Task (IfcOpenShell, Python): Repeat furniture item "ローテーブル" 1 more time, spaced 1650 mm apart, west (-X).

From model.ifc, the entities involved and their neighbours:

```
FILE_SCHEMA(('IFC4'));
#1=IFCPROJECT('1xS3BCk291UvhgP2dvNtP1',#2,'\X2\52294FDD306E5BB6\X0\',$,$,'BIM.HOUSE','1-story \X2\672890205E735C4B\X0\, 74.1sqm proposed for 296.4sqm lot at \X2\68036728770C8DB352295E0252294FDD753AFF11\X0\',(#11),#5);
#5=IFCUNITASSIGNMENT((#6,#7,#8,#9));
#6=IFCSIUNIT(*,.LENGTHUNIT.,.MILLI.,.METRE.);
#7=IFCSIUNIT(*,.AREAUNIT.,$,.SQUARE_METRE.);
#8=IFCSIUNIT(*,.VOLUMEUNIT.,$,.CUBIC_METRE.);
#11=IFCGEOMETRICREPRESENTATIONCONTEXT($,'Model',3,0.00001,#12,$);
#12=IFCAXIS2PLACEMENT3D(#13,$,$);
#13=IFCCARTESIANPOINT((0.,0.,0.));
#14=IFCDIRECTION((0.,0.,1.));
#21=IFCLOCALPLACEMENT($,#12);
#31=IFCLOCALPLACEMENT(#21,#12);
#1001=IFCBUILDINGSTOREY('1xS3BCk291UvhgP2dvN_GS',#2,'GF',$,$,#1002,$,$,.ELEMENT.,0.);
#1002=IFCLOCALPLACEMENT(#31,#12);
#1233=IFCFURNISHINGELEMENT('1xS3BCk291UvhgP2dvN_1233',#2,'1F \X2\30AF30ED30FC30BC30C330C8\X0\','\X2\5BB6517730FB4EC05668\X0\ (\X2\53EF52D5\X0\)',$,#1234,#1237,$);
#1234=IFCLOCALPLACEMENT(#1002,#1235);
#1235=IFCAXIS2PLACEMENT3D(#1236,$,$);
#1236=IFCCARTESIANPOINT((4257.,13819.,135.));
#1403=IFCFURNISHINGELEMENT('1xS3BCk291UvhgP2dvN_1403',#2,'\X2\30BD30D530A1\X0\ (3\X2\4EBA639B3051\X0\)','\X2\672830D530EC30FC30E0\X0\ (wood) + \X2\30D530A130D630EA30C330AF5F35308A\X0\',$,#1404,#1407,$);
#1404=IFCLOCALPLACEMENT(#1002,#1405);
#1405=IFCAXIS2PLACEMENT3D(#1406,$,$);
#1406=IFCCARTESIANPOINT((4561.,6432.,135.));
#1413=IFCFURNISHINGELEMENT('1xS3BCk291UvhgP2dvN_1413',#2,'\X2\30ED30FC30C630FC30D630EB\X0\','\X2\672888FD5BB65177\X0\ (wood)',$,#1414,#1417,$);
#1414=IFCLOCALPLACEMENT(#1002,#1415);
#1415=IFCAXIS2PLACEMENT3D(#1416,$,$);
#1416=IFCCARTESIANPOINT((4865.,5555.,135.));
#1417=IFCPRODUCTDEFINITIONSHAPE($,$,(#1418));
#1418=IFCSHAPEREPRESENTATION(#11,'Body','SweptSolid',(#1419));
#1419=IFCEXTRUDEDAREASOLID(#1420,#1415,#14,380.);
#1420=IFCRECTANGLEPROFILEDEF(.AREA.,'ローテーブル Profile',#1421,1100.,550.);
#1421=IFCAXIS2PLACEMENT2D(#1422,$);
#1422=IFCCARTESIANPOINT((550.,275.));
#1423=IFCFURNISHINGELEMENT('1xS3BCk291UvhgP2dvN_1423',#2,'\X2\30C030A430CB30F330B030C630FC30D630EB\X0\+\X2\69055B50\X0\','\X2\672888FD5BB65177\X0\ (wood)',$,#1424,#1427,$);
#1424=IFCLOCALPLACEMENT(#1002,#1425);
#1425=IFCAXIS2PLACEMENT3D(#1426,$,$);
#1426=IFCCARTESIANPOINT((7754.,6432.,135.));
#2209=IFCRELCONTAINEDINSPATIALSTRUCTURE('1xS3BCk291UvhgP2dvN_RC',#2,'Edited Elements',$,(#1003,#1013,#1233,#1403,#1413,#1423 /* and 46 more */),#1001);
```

```python
import numpy as np
import ifcopenshell
import ifcopenshell.api.geometry
import ifcopenshell.api.root
import ifcopenshell.util.element
import ifcopenshell.util.placement

model = ifcopenshell.open("model.ifc")


def reuse_history(source, copy):
    """copy_class also copies each property set's owner history, people and application; keep the originals."""
    for rel in copy.IsDefinedBy:
        if rel.is_a("IfcRelDefinesByProperties") and (history := rel.RelatingPropertyDefinition.OwnerHistory):
            rel.RelatingPropertyDefinition.OwnerHistory = source.OwnerHistory
            ifcopenshell.util.element.remove_deep2(model, history)


source = model.by_guid("1xS3BCk291UvhgP2dvN_1413")
base = ifcopenshell.util.placement.get_local_placement(source.ObjectPlacement)
step = np.array([-1.0, 0.0, 0.0]) * 1650.0

for i in range(1, 2):
    copy = ifcopenshell.api.root.copy_class(model, product=source)
    copy.Representation = ifcopenshell.util.element.copy_deep(
        model, source.Representation, exclude=["IfcGeometricRepresentationContext", "IfcRepresentationMap"]
    )
    reuse_history(source, copy)
    matrix = base.copy()
    matrix[:3, 3] += i * step
    print("added at", matrix[:3, 3].round(3) + 0.0)
    ifcopenshell.api.geometry.edit_object_placement(model, product=copy, matrix=matrix, is_si=False)

model.write("model_updated.ifc")
```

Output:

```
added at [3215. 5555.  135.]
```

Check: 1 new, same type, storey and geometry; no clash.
